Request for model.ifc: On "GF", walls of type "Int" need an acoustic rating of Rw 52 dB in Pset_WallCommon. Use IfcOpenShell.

First a look at what the model holds.

```python
import ifcopenshell
import ifcopenshell.util.element

model = ifcopenshell.open("model.ifc")
print(model.schema)
storey = next(s for s in model.by_type("IfcBuildingStorey") if s.Name == "GF")
walls = [e for e in ifcopenshell.util.element.get_decomposition(storey) if e.is_a("IfcWall")]
seen = {}
for e in walls:
    element_type = ifcopenshell.util.element.get_type(e)
    key = (element_type.Name if element_type != e and element_type else None, ifcopenshell.util.element.get_pset(e, "Pset_WallCommon", "AcousticRating"))
    seen[key] = seen.get(key, 0) + 1
for (name, value), count in sorted(seen.items(), key=str):
    print(count, "x", name, "|", value)
```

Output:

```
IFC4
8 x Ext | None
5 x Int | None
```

```python
import ifcopenshell
import ifcopenshell.api.pset
import ifcopenshell.util.element

model = ifcopenshell.open("model.ifc")

storey = next(s for s in model.by_type("IfcBuildingStorey") if s.Name == "GF")
walls = [e for e in ifcopenshell.util.element.get_decomposition(storey) if e.is_a("IfcWall")]

count = 0
for e in walls:
    element_type = ifcopenshell.util.element.get_type(e)
    if element_type in (None, e) or element_type.Name != "Int":
        continue
    # add_pset returns the element's existing set when there is one.
    pset = ifcopenshell.api.pset.add_pset(model, product=e, name="Pset_WallCommon")
    ifcopenshell.api.pset.edit_pset(model, pset=pset, properties={"AcousticRating": "Rw 52 dB"})
    count += 1

print(count, "walls updated")

model.write("model_edited.ifc")
```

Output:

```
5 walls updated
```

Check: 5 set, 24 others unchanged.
